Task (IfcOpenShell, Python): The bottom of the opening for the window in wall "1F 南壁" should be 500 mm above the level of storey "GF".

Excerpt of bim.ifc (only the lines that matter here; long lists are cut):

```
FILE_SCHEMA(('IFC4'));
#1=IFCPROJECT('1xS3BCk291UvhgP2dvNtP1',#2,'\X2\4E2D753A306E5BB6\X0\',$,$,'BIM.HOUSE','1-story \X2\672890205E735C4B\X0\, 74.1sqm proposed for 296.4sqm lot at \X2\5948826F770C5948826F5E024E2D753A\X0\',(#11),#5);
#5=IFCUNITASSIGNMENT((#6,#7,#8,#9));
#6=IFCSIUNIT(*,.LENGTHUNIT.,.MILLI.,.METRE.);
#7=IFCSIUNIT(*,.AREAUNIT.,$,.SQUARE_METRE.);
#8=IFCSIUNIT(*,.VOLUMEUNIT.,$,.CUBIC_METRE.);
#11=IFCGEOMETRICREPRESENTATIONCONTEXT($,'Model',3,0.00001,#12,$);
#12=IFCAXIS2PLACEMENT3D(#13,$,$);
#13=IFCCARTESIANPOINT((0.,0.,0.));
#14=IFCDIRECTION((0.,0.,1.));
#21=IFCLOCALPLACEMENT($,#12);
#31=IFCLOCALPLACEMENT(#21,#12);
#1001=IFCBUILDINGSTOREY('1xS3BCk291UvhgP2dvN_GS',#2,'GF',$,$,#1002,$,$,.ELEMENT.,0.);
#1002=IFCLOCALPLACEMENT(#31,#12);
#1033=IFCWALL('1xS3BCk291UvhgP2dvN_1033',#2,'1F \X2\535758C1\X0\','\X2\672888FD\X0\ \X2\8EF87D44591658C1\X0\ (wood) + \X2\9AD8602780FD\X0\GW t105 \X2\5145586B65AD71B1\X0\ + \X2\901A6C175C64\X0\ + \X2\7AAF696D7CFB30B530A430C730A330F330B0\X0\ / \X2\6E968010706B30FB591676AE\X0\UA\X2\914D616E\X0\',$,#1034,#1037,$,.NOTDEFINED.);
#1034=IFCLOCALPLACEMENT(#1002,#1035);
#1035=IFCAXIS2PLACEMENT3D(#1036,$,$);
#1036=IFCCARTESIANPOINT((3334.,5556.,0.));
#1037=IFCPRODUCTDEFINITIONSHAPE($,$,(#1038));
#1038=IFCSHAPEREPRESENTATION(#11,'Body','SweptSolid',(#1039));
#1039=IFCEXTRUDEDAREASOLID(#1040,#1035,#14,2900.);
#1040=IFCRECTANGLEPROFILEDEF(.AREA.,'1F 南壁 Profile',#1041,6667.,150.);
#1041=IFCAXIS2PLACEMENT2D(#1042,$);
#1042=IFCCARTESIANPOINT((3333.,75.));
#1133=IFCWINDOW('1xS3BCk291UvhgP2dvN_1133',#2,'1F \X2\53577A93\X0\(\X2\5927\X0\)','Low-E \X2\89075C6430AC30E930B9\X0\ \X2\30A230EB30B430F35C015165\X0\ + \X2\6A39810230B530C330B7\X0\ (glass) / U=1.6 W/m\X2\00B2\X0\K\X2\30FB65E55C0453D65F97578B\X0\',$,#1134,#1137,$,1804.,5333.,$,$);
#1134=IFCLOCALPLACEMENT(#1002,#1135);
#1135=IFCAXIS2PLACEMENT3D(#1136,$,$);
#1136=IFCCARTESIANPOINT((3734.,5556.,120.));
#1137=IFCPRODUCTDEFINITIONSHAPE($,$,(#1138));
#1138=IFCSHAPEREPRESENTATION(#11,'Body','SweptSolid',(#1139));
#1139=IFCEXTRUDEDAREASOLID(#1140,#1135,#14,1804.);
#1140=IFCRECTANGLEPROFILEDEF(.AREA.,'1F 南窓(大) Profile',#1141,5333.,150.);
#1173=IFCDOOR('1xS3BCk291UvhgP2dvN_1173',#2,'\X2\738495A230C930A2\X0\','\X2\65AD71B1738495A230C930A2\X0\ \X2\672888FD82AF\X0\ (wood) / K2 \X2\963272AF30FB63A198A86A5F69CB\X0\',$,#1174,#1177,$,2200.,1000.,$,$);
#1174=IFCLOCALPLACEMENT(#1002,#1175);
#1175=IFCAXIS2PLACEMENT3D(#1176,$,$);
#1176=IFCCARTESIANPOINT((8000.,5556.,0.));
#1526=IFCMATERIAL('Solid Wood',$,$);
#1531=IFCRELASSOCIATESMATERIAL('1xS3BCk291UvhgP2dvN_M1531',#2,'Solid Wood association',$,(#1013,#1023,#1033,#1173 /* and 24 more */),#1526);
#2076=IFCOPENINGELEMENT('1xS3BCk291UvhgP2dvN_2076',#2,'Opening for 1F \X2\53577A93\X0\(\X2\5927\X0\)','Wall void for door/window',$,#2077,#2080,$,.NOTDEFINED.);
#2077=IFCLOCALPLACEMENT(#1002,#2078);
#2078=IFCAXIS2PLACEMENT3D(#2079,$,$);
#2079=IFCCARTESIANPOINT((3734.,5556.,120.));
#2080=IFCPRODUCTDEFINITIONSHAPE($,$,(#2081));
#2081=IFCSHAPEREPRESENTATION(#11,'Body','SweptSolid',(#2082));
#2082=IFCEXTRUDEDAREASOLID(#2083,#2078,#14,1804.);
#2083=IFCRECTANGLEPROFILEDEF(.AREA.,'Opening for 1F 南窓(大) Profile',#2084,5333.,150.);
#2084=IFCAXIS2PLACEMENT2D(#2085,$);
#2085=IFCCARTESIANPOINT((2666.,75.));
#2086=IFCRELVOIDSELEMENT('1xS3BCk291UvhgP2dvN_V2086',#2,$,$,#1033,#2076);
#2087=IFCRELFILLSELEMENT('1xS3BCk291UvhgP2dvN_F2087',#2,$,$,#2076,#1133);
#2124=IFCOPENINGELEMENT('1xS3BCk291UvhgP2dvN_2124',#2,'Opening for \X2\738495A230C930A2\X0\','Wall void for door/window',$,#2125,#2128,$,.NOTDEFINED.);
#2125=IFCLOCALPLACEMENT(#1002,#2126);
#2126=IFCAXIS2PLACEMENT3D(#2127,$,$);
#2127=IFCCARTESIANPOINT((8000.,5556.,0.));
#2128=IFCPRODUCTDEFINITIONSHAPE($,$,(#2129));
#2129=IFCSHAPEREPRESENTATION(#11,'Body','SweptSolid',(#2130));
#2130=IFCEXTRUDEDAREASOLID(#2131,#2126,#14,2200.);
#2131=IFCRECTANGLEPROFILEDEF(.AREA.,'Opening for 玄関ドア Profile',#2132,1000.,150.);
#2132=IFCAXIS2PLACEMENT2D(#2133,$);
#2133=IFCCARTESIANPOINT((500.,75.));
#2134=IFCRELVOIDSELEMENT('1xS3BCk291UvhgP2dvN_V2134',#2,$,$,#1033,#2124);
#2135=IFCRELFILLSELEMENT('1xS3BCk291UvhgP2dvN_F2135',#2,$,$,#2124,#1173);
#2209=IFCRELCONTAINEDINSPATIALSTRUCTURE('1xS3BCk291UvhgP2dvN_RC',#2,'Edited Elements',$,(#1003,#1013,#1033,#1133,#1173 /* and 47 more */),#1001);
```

```python
import numpy as np
import ifcopenshell
import ifcopenshell.api.geometry
import ifcopenshell.geom
import ifcopenshell.util.element
import ifcopenshell.util.placement
import ifcopenshell.util.shape
import ifcopenshell.util.unit

model = ifcopenshell.open("bim.ifc")
unit_scale = ifcopenshell.util.unit.calculate_unit_scale(model)

window = model.by_id(1133)
opening = window.FillsVoids[0].RelatingOpeningElement
storey = ifcopenshell.util.element.get_container(window, ifc_class="IfcBuildingStorey")
level = ifcopenshell.util.placement.get_local_placement(storey.ObjectPlacement)[2, 3]

# The opening's origin need not be at the sill, so measure its lowest point.
shape = ifcopenshell.geom.create_shape(ifcopenshell.geom.settings(), opening)
bottom = ifcopenshell.util.shape.get_shape_bottom_elevation(shape, shape.geometry) / unit_scale
dz = level + 0.5 / unit_scale - bottom

shift = np.array([0.0, 0.0, dz])
# The window is not placed relative to its opening, so move both.
for product in (opening, window):
    matrix = ifcopenshell.util.placement.get_local_placement(product.ObjectPlacement)
    matrix[:3, 3] += shift
    ifcopenshell.api.geometry.edit_object_placement(model, product=product, matrix=matrix, is_si=False)

print(f"moved by {dz * unit_scale:+.3f} m")

model.write("bim_edited.ifc")
```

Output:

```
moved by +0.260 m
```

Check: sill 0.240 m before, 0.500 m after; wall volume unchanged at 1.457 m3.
